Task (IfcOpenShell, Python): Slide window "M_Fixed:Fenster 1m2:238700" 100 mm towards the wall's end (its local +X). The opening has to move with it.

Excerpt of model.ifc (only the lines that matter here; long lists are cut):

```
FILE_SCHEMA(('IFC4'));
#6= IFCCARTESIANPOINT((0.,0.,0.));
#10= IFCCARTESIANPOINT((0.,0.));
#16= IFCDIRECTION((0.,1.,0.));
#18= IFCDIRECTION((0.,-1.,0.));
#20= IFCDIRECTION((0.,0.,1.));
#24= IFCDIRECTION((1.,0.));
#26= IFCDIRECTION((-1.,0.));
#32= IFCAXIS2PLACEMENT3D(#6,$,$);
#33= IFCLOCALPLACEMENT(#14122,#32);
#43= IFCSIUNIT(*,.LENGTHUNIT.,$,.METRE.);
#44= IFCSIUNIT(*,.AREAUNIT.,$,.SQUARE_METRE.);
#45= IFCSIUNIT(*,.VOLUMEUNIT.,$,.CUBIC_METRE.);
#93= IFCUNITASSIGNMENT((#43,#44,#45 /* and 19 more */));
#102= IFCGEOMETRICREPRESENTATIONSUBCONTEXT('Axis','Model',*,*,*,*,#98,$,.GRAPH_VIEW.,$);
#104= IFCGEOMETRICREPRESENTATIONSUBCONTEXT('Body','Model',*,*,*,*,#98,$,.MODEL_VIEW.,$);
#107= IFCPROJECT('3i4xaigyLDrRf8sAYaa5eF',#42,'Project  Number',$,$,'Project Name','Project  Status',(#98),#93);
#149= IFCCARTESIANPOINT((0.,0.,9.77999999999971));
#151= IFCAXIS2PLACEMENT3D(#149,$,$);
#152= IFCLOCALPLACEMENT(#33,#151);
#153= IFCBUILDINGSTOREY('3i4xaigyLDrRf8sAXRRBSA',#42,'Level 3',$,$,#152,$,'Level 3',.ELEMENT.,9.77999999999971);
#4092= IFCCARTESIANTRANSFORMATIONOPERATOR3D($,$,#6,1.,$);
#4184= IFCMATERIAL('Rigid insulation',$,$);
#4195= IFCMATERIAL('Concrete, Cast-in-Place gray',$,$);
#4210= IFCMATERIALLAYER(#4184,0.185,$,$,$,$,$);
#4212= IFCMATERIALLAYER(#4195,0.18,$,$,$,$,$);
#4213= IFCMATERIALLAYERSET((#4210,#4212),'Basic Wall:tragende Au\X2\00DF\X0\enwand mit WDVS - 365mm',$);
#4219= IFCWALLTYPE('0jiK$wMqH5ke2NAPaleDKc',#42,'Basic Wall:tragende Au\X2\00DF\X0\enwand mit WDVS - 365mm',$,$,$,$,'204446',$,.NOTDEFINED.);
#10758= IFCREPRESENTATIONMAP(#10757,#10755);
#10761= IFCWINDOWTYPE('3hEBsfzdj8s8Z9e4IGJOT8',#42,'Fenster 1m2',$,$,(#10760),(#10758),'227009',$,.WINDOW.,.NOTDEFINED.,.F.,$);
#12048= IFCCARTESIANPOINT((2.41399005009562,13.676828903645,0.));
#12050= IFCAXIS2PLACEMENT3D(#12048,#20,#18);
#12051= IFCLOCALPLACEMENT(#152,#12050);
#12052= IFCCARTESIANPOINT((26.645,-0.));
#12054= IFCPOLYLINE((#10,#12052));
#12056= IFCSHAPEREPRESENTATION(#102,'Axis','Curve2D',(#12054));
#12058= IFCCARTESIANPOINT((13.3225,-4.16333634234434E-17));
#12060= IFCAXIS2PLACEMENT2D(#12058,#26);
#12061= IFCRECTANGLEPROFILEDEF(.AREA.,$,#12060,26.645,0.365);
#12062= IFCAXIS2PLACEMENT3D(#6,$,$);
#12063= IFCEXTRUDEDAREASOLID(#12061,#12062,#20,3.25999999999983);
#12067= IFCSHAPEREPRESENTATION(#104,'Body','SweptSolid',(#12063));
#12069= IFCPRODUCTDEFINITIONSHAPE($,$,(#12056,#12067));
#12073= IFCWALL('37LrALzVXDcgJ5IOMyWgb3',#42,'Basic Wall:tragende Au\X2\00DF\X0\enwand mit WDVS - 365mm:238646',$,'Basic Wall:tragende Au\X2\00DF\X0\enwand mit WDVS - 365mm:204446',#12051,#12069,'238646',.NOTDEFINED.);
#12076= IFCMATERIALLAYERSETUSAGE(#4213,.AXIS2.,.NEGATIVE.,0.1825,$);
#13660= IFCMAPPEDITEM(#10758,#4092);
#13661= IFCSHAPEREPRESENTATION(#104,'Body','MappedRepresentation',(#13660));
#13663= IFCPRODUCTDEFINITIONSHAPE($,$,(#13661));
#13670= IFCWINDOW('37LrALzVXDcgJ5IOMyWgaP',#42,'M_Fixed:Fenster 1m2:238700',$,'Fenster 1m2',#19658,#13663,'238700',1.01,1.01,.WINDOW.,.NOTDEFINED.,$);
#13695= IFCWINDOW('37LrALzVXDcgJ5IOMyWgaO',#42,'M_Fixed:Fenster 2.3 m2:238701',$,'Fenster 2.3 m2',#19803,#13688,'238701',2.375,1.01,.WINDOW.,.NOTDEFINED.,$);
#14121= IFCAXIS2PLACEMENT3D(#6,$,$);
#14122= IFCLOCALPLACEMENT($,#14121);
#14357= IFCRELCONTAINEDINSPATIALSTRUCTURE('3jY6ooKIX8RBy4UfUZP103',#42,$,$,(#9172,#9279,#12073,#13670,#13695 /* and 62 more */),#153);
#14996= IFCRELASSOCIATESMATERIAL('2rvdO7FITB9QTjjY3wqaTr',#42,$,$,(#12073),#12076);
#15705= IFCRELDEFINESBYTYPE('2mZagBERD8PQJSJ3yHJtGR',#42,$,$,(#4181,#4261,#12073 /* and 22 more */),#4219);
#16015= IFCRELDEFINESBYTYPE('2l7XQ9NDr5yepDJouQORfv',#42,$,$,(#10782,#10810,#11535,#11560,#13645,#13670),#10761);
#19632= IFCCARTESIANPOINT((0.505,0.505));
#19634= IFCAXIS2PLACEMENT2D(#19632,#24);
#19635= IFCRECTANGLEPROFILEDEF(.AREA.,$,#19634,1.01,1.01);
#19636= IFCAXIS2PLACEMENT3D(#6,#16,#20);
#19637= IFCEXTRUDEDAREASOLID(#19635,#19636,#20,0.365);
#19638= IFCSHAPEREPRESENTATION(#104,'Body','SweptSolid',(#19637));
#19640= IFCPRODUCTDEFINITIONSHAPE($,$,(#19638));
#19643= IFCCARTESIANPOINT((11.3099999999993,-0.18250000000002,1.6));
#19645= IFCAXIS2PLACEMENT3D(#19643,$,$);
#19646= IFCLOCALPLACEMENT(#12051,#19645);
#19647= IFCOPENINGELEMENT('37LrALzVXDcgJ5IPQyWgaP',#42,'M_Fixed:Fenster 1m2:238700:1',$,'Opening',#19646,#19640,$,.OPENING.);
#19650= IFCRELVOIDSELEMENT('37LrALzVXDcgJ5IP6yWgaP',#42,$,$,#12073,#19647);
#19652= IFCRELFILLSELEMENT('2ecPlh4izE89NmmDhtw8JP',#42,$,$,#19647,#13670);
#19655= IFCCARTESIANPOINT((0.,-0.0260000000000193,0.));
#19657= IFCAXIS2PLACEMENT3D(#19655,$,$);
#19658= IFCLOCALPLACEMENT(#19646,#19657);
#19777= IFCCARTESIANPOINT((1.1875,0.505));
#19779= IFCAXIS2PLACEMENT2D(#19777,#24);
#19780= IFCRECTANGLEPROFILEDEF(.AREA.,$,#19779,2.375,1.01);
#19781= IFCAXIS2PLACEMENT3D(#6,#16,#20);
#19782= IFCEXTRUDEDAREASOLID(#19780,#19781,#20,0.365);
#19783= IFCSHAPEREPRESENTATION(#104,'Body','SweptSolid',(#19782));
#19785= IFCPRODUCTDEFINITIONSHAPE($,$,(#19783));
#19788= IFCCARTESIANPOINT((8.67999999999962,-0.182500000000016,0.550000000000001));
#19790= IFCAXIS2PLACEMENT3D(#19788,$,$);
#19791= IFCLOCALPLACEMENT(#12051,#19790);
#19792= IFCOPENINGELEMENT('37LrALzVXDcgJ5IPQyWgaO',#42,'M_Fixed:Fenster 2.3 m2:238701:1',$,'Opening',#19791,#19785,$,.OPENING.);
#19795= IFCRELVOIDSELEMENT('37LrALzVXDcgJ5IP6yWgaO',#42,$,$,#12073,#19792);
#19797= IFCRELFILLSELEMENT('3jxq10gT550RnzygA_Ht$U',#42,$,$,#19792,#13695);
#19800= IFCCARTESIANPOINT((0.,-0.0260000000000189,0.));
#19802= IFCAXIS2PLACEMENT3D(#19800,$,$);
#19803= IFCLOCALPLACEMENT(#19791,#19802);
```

```python
import ifcopenshell
import ifcopenshell.api.geometry
import ifcopenshell.util.placement
import ifcopenshell.util.unit

model = ifcopenshell.open("model.ifc")
unit_scale = ifcopenshell.util.unit.calculate_unit_scale(model)

window = model.by_guid("37LrALzVXDcgJ5IOMyWgaP")
opening = window.FillsVoids[0].RelatingOpeningElement
wall = opening.VoidsElements[0].RelatingBuildingElement

wall_matrix = ifcopenshell.util.placement.get_local_placement(wall.ObjectPlacement)
shift = wall_matrix[:3, 0] * 0.1 / unit_scale
before = ifcopenshell.util.placement.get_local_placement(window.ObjectPlacement)[:3, 3].copy()

# The window is placed relative to its opening, so it follows when the opening moves.
matrix = ifcopenshell.util.placement.get_local_placement(opening.ObjectPlacement)
matrix[:3, 3] += shift
ifcopenshell.api.geometry.edit_object_placement(
    model, product=opening, matrix=matrix, is_si=False, should_transform_children=True
)

after = ifcopenshell.util.placement.get_local_placement(window.ObjectPlacement)[:3, 3]
print("window moved by", (after - before).round(3) + 0.0)

model.write("model-out.ifc")
```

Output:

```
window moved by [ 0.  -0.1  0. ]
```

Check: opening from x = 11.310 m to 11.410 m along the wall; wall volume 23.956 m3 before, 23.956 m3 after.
